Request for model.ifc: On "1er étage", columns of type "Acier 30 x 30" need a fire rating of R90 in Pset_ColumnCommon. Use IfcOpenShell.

First a look at what the model holds.

```python
import ifcopenshell
import ifcopenshell.util.element

model = ifcopenshell.open("model.ifc")
print(model.schema)
storey = next(s for s in model.by_type("IfcBuildingStorey") if s.Name == "1er étage")
columns = [e for e in ifcopenshell.util.element.get_decomposition(storey) if e.is_a("IfcColumn")]
seen = {}
for e in columns:
    element_type = ifcopenshell.util.element.get_type(e)
    key = (element_type.Name if element_type != e and element_type else None, ifcopenshell.util.element.get_pset(e, "Pset_ColumnCommon", "FireRating"))
    seen[key] = seen.get(key, 0) + 1
for (name, value), count in sorted(seen.items(), key=str):
    print(count, "x", name, "|", value)
```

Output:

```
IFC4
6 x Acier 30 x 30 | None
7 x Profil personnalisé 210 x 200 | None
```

```python
import ifcopenshell
import ifcopenshell.api.pset
import ifcopenshell.util.element

model = ifcopenshell.open("model.ifc")

storey = next(s for s in model.by_type("IfcBuildingStorey") if s.Name == "1er étage")
columns = [e for e in ifcopenshell.util.element.get_decomposition(storey) if e.is_a("IfcColumn")]

count = 0
for e in columns:
    element_type = ifcopenshell.util.element.get_type(e)
    if element_type in (None, e) or element_type.Name != "Acier 30 x 30":
        continue
    # add_pset returns the element's existing set when there is one.
    pset = ifcopenshell.api.pset.add_pset(model, product=e, name="Pset_ColumnCommon")
    ifcopenshell.api.pset.edit_pset(model, pset=pset, properties={"FireRating": "R90"})
    count += 1

print(count, "columns updated")

model.write("model_updated.ifc")
```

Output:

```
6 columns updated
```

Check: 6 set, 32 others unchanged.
